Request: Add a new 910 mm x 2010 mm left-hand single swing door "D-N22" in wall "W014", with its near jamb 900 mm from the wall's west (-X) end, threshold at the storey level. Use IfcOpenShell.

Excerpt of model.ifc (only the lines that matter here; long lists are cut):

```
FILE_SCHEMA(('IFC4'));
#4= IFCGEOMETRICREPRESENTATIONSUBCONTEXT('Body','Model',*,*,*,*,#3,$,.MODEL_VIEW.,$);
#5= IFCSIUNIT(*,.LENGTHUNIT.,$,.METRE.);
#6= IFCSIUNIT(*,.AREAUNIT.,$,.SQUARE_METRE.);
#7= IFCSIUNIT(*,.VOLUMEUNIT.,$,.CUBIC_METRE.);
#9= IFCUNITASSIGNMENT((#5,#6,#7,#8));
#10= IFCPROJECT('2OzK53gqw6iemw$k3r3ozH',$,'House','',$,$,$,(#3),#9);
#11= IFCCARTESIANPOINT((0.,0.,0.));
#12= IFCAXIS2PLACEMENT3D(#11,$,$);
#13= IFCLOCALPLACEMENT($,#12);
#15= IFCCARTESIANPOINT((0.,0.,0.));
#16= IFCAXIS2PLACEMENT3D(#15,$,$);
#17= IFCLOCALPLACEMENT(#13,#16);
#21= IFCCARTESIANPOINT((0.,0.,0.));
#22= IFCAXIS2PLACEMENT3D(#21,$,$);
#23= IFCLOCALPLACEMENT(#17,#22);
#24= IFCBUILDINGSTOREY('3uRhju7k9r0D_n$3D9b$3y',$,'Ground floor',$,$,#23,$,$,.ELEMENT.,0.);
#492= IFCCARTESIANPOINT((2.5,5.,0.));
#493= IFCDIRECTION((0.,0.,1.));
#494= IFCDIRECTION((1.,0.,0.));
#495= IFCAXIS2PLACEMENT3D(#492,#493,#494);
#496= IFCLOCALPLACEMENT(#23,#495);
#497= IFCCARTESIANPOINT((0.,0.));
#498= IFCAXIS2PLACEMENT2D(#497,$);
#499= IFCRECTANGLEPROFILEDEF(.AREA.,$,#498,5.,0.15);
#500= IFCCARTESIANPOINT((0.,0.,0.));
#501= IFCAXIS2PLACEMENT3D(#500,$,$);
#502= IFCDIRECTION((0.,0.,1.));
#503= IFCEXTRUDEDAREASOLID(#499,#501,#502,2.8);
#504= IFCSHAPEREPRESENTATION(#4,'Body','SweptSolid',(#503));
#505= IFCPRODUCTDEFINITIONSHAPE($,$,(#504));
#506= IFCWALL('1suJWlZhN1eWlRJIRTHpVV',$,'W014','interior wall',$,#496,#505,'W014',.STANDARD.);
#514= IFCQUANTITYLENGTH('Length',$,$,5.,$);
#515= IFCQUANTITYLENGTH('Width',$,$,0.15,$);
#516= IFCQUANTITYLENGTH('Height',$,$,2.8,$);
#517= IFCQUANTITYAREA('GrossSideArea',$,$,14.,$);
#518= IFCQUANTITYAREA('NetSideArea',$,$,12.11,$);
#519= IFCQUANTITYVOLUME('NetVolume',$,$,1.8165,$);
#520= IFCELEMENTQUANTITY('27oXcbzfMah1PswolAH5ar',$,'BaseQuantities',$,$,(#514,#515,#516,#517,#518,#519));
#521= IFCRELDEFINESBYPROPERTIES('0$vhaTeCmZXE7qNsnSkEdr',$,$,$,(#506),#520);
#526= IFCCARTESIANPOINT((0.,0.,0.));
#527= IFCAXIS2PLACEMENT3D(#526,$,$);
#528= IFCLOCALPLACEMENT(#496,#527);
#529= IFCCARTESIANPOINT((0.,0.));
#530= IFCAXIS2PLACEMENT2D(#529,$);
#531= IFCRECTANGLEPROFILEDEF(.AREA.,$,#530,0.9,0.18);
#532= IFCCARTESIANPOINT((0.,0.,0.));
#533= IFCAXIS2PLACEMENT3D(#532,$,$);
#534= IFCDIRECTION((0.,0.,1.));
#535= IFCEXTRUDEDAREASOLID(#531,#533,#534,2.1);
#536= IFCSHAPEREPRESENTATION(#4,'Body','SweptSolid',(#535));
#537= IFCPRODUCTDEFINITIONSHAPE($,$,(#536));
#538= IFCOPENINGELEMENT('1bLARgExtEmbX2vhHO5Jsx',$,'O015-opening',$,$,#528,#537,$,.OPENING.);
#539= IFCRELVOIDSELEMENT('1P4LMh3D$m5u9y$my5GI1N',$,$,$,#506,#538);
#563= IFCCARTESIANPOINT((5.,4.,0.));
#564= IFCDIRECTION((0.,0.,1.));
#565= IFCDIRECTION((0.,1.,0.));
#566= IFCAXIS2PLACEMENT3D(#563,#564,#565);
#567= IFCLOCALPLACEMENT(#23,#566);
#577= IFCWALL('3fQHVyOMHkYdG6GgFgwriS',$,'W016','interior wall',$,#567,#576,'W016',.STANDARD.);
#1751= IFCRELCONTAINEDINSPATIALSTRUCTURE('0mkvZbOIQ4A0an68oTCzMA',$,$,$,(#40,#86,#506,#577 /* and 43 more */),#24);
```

```python
import numpy as np
import ifcopenshell
import ifcopenshell.api.feature
import ifcopenshell.api.geometry
import ifcopenshell.api.pset
import ifcopenshell.api.root
import ifcopenshell.api.spatial
import ifcopenshell.geom
import ifcopenshell.util.element
import ifcopenshell.util.placement
import ifcopenshell.util.representation
import ifcopenshell.util.shape
import ifcopenshell.util.unit

model = ifcopenshell.open("model.ifc")
unit_scale = ifcopenshell.util.unit.calculate_unit_scale(model)
area_scale = ifcopenshell.util.unit.calculate_unit_scale(model, "AREAUNIT")
volume_scale = ifcopenshell.util.unit.calculate_unit_scale(model, "VOLUMEUNIT")
settings = ifcopenshell.geom.settings()


def volume(element):
    """Net volume in cubic metres, openings subtracted."""
    shape = ifcopenshell.geom.create_shape(settings, element)
    return ifcopenshell.util.shape.get_volume(shape.geometry)


wall = model.by_guid("1suJWlZhN1eWlRJIRTHpVV")
storey = ifcopenshell.util.element.get_container(wall, ifc_class="IfcBuildingStorey")
context = ifcopenshell.util.representation.get_context(model, "Model", "Body", "MODEL_VIEW")
before = volume(wall)

width, height, from_end, sill = 0.91, 2.01, 0.9, 0.0  # metres

# The wall runs along its own X axis, and the end named is its -X end.
wall_shape = ifcopenshell.geom.create_shape(settings, wall)
x, y, z = ifcopenshell.util.shape.get_vertices(wall_shape.geometry).T
start = x.min() + from_end
face, thickness = float(y.min()), float(y.max() - y.min())
wall_matrix = ifcopenshell.util.placement.get_local_placement(wall.ObjectPlacement)
level = ifcopenshell.util.placement.get_local_placement(storey.ObjectPlacement)[2, 3]


def in_wall(x, y):
    """Placement at x, y metres in the wall's axes, at sill height."""
    matrix = wall_matrix.copy()
    matrix[:, 3] = wall_matrix @ np.array([x / unit_scale, y / unit_scale, 0.0, 1.0])
    matrix[2, 3] = level + sill / unit_scale
    return matrix


# Opening: a box that overshoots both wall faces by 50 mm.
opening = ifcopenshell.api.root.create_entity(model, ifc_class="IfcOpeningElement", predefined_type="OPENING")
box = ifcopenshell.api.geometry.add_wall_representation(
    model, context=context, length=width, height=height, thickness=thickness + 0.1
)
ifcopenshell.api.geometry.assign_representation(model, product=opening, representation=box)
ifcopenshell.api.geometry.edit_object_placement(model, product=opening, matrix=in_wall(start, face - 0.05), is_si=False)
ifcopenshell.api.feature.add_feature(model, feature=opening, element=wall)

door = ifcopenshell.api.root.create_entity(model, ifc_class="IfcDoor", name="D-N22", predefined_type="DOOR")
door.OverallWidth, door.OverallHeight = width / unit_scale, height / unit_scale
door.OperationType = "SINGLE_SWING_LEFT"
body = ifcopenshell.api.geometry.add_door_representation(
    model,
    context=context,
    overall_width=door.OverallWidth,
    overall_height=door.OverallHeight,
    operation_type="SINGLE_SWING_LEFT",
    lining_properties={"LiningDepth": thickness / unit_scale, "ThresholdDepth": thickness / unit_scale},
)
ifcopenshell.api.geometry.assign_representation(model, product=door, representation=body)
ifcopenshell.api.spatial.assign_container(model, products=[door], relating_structure=storey)
ifcopenshell.api.feature.add_filling(model, opening=opening, element=door)

# The lining spans the wall, so the door starts at the wall face.
ifcopenshell.api.geometry.edit_object_placement(model, product=door, matrix=in_wall(start, face), is_si=False)

after = volume(wall)

# Update the wall's stored quantities.
qto = model.by_id(ifcopenshell.util.element.get_pset(wall, "BaseQuantities", should_inherit=False)["id"])
ifcopenshell.api.pset.edit_qto(model, qto=qto, properties={
    "NetSideArea": after / thickness / area_scale,
    "NetVolume": after / volume_scale,
})

print(f"wall volume {before:.3f} -> {after:.3f} m3")

model.write("model_v2.ifc")
```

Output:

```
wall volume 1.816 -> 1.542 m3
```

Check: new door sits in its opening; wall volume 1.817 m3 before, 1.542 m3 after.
